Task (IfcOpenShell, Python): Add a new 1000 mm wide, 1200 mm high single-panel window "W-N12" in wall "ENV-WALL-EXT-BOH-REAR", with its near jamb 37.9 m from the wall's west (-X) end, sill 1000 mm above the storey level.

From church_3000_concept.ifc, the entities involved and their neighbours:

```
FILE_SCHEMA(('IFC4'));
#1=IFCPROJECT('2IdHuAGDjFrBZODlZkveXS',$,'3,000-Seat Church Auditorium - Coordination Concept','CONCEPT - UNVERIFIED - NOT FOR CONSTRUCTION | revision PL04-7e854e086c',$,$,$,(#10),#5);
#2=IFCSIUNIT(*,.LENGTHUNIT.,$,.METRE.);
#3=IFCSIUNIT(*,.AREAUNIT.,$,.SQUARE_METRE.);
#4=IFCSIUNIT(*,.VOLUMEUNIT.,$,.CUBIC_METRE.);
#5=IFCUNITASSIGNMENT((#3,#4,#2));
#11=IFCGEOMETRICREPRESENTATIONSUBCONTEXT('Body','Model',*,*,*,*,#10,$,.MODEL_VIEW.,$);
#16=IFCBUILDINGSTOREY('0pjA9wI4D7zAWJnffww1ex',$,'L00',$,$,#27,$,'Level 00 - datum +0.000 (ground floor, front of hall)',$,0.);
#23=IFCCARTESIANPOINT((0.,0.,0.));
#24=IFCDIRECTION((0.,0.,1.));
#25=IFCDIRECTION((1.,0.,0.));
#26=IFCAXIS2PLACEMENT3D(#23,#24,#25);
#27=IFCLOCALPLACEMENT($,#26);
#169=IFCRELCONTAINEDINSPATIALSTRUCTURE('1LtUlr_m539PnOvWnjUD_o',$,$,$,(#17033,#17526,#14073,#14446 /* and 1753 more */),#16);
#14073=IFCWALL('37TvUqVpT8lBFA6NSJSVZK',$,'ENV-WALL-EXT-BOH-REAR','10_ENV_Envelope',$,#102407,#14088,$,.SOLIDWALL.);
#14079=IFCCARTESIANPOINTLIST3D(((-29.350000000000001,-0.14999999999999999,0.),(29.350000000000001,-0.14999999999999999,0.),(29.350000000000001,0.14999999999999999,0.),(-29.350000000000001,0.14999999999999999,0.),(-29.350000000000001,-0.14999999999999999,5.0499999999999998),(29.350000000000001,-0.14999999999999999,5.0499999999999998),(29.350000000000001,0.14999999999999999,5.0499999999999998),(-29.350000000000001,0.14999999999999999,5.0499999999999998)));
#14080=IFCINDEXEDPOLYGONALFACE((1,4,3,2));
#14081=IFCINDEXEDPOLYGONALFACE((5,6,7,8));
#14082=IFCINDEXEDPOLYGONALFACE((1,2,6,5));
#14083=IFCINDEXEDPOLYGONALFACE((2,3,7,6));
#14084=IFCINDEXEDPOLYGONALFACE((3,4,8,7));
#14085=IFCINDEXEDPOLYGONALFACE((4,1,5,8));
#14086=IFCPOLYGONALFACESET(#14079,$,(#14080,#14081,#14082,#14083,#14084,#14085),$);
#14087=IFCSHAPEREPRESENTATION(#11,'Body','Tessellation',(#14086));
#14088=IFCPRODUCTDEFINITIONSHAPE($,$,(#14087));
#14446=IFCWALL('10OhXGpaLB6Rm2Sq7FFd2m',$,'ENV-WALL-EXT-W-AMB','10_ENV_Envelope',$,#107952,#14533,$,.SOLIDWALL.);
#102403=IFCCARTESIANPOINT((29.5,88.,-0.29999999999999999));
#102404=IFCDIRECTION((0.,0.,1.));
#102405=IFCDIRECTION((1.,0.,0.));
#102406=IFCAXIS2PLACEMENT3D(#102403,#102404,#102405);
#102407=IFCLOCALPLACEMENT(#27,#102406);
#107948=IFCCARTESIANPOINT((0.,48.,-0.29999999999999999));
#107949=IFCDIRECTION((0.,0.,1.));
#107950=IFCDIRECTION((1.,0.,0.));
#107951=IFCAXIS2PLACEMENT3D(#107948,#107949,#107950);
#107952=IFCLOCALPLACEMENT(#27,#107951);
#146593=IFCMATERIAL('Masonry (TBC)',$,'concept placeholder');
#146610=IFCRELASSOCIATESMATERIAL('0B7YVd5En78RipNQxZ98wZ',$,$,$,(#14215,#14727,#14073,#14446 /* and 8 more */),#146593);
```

```python
import numpy as np
import ifcopenshell
import ifcopenshell.api.feature
import ifcopenshell.api.geometry
import ifcopenshell.api.root
import ifcopenshell.api.spatial
import ifcopenshell.geom
import ifcopenshell.util.element
import ifcopenshell.util.placement
import ifcopenshell.util.representation
import ifcopenshell.util.shape
import ifcopenshell.util.unit

model = ifcopenshell.open("church_3000_concept.ifc")
unit_scale = ifcopenshell.util.unit.calculate_unit_scale(model)
settings = ifcopenshell.geom.settings()


def volume(element):
    """Net volume in cubic metres, openings subtracted."""
    shape = ifcopenshell.geom.create_shape(settings, element)
    return ifcopenshell.util.shape.get_volume(shape.geometry)


wall = model.by_id(14073)
storey = ifcopenshell.util.element.get_container(wall, ifc_class="IfcBuildingStorey")
context = ifcopenshell.util.representation.get_context(model, "Model", "Body", "MODEL_VIEW")
before = volume(wall)

width, height, from_end, sill = 1, 1.2, 37.9, 1  # metres

# The wall runs along its own X axis, and the end named is its -X end.
wall_shape = ifcopenshell.geom.create_shape(settings, wall)
x, y, z = ifcopenshell.util.shape.get_vertices(wall_shape.geometry).T
start = x.min() + from_end
face, thickness = float(y.min()), float(y.max() - y.min())
wall_matrix = ifcopenshell.util.placement.get_local_placement(wall.ObjectPlacement)
level = ifcopenshell.util.placement.get_local_placement(storey.ObjectPlacement)[2, 3]


def in_wall(x, y):
    """Placement at x, y metres in the wall's axes, at sill height."""
    matrix = wall_matrix.copy()
    matrix[:, 3] = wall_matrix @ np.array([x / unit_scale, y / unit_scale, 0.0, 1.0])
    matrix[2, 3] = level + sill / unit_scale
    return matrix


# Opening: a box that overshoots both wall faces by 50 mm.
opening = ifcopenshell.api.root.create_entity(model, ifc_class="IfcOpeningElement", predefined_type="OPENING")
box = ifcopenshell.api.geometry.add_wall_representation(
    model, context=context, length=width, height=height, thickness=thickness + 0.1
)
ifcopenshell.api.geometry.assign_representation(model, product=opening, representation=box)
ifcopenshell.api.geometry.edit_object_placement(model, product=opening, matrix=in_wall(start, face - 0.05), is_si=False)
ifcopenshell.api.feature.add_feature(model, feature=opening, element=wall)

window = ifcopenshell.api.root.create_entity(model, ifc_class="IfcWindow", name="W-N12", predefined_type="WINDOW")
window.OverallWidth, window.OverallHeight = width / unit_scale, height / unit_scale
window.PartitioningType = "SINGLE_PANEL"
body = ifcopenshell.api.geometry.add_window_representation(
    model,
    context=context,
    overall_width=window.OverallWidth,
    overall_height=window.OverallHeight,
    partition_type="SINGLE_PANEL",
)
ifcopenshell.api.geometry.assign_representation(model, product=window, representation=body)
ifcopenshell.api.spatial.assign_container(model, products=[window], relating_structure=storey)
ifcopenshell.api.feature.add_filling(model, opening=opening, element=window)

# Centre the window in the wall's thickness.
ifcopenshell.api.geometry.edit_object_placement(model, product=window, matrix=in_wall(start, face), is_si=False)
window_shape = ifcopenshell.geom.create_shape(settings, window)
depth = ifcopenshell.util.shape.get_vertices(window_shape.geometry)[:, 1]
offset = face + thickness / 2 - (depth.min() + depth.max()) / 2
ifcopenshell.api.geometry.edit_object_placement(model, product=window, matrix=in_wall(start, offset), is_si=False)

after = volume(wall)

print(f"wall volume {before:.3f} -> {after:.3f} m3")

model.write("church_3000_concept-out.ifc")
```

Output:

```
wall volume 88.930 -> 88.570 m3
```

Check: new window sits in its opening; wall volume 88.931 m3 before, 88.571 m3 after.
